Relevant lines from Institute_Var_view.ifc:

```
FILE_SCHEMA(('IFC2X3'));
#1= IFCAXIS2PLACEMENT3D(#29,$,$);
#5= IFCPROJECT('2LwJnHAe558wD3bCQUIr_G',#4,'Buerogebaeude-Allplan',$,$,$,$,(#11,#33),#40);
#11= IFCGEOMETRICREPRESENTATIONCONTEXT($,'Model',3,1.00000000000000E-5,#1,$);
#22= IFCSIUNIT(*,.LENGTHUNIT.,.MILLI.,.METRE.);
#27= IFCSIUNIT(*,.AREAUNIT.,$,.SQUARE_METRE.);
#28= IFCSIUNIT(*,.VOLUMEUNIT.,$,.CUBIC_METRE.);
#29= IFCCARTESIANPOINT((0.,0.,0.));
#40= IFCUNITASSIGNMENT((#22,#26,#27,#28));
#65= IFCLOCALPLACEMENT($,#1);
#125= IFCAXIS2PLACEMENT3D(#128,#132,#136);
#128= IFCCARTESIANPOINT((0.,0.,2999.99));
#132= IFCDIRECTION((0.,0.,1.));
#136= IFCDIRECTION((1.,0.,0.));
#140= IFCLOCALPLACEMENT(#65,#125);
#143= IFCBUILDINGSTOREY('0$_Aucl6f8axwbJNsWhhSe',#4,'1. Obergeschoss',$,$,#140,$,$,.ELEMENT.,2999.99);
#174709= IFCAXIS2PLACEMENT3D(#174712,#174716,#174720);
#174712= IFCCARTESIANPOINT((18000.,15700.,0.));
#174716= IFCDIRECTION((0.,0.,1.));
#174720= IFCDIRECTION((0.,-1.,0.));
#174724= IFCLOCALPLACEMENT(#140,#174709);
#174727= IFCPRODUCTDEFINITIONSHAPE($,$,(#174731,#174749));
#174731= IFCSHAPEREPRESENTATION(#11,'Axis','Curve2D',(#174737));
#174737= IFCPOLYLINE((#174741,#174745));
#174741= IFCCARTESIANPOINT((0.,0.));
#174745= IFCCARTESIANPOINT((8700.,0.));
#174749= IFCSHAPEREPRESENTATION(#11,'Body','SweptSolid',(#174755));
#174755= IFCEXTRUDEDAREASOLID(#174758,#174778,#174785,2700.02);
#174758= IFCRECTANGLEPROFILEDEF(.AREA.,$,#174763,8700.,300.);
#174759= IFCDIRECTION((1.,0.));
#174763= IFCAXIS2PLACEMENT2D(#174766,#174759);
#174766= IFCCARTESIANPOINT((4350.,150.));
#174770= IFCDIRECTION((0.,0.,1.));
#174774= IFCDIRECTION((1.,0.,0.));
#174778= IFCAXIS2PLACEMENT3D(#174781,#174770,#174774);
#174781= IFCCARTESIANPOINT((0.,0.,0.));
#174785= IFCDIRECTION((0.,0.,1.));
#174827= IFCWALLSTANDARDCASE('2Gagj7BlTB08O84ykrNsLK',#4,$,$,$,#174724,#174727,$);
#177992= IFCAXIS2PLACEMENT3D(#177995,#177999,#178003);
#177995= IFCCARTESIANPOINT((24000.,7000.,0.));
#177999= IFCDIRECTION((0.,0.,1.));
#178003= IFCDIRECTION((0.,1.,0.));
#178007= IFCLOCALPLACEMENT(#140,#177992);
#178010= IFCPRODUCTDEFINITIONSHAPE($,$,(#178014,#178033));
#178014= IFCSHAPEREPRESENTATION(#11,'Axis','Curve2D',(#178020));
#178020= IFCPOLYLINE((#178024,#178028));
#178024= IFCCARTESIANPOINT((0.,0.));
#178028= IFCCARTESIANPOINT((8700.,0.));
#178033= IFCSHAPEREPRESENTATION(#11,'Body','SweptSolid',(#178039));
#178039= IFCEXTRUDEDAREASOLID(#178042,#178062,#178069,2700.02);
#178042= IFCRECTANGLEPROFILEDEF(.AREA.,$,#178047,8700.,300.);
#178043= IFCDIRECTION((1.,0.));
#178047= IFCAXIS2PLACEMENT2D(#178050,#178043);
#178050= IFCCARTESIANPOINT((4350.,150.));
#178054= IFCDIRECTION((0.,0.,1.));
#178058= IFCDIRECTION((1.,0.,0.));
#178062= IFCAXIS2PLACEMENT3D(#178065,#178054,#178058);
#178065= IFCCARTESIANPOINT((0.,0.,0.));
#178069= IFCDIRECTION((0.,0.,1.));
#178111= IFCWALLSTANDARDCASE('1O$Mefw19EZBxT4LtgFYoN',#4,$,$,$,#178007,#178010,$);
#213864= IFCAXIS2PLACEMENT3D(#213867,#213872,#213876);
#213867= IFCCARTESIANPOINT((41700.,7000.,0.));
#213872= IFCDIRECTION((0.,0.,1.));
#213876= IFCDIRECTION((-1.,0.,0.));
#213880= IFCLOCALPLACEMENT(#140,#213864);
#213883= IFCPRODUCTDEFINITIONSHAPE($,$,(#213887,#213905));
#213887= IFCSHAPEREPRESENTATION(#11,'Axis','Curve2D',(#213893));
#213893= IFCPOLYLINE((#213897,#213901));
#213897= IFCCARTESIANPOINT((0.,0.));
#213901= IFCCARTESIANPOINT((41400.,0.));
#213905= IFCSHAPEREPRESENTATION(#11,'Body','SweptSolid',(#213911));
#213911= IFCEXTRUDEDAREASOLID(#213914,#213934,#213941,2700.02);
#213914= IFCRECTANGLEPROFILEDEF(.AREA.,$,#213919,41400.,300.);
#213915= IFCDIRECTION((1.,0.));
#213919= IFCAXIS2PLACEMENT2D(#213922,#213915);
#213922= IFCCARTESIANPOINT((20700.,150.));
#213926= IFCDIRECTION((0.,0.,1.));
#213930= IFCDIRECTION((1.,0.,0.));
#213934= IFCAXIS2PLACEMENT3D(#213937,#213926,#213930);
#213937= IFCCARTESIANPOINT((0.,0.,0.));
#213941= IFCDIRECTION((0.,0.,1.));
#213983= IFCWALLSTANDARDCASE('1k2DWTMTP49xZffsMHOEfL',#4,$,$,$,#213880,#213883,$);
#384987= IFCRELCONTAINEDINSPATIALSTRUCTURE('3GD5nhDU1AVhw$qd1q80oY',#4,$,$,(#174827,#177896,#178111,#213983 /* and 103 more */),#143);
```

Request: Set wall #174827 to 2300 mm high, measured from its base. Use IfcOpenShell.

```python
import ifcopenshell
import ifcopenshell.geom
import ifcopenshell.util.shape

model = ifcopenshell.open("Institute_Var_view.ifc")
settings = ifcopenshell.geom.settings()


def volume(element):
    """Net volume in cubic metres, openings subtracted."""
    shape = ifcopenshell.geom.create_shape(settings, element)
    return ifcopenshell.util.shape.get_volume(shape.geometry)


wall = model.by_id(174827)
before = volume(wall)

body = next(r for r in wall.Representation.Representations if r.RepresentationIdentifier == "Body")
solid = body.Items[0]
old_height = solid.Depth
solid.Depth = 2300.0
after = volume(wall)

print(f"height {old_height:g} -> {solid.Depth:g}, volume {before:.3f} -> {after:.3f} m3")

model.write("Institute_Var_view_rev.ifc")
```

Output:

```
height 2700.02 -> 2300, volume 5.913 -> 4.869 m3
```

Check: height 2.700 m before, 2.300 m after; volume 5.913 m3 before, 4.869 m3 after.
